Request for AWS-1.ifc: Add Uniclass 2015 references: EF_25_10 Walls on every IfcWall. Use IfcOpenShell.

First a look at what the model holds.

```python
import ifcopenshell

model = ifcopenshell.open("AWS-1.ifc")
print(model.schema)
print("classifications:", [c.Name for c in model.by_type("IfcClassification")])
for ifc_class in ("IfcDoor", "IfcRoof", "IfcStair", "IfcWall", "IfcWindow"):
    print(ifc_class, len(model.by_type(ifc_class)))
```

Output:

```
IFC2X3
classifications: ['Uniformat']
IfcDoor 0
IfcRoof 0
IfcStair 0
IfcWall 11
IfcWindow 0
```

```python
import ifcopenshell
import ifcopenshell.api.classification

model = ifcopenshell.open("AWS-1.ifc")

# IFC2X3 requires Source and Edition and has no link from the project to the system.
system = model.create_entity("IfcClassification", Source="NBS", Edition="2015", Name="Uniclass 2015")

codes = {
    "IfcWall": ("EF_25_10", "Walls"),
}
for ifc_class, (code, name) in codes.items():
    products = model.by_type(ifc_class)
    ifcopenshell.api.classification.add_reference(
        model, products=products, classification=system, identification=code, name=name
    )
    print(code, len(products))

model.write("AWS-1-out.ifc")
```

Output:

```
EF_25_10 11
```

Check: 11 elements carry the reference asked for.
